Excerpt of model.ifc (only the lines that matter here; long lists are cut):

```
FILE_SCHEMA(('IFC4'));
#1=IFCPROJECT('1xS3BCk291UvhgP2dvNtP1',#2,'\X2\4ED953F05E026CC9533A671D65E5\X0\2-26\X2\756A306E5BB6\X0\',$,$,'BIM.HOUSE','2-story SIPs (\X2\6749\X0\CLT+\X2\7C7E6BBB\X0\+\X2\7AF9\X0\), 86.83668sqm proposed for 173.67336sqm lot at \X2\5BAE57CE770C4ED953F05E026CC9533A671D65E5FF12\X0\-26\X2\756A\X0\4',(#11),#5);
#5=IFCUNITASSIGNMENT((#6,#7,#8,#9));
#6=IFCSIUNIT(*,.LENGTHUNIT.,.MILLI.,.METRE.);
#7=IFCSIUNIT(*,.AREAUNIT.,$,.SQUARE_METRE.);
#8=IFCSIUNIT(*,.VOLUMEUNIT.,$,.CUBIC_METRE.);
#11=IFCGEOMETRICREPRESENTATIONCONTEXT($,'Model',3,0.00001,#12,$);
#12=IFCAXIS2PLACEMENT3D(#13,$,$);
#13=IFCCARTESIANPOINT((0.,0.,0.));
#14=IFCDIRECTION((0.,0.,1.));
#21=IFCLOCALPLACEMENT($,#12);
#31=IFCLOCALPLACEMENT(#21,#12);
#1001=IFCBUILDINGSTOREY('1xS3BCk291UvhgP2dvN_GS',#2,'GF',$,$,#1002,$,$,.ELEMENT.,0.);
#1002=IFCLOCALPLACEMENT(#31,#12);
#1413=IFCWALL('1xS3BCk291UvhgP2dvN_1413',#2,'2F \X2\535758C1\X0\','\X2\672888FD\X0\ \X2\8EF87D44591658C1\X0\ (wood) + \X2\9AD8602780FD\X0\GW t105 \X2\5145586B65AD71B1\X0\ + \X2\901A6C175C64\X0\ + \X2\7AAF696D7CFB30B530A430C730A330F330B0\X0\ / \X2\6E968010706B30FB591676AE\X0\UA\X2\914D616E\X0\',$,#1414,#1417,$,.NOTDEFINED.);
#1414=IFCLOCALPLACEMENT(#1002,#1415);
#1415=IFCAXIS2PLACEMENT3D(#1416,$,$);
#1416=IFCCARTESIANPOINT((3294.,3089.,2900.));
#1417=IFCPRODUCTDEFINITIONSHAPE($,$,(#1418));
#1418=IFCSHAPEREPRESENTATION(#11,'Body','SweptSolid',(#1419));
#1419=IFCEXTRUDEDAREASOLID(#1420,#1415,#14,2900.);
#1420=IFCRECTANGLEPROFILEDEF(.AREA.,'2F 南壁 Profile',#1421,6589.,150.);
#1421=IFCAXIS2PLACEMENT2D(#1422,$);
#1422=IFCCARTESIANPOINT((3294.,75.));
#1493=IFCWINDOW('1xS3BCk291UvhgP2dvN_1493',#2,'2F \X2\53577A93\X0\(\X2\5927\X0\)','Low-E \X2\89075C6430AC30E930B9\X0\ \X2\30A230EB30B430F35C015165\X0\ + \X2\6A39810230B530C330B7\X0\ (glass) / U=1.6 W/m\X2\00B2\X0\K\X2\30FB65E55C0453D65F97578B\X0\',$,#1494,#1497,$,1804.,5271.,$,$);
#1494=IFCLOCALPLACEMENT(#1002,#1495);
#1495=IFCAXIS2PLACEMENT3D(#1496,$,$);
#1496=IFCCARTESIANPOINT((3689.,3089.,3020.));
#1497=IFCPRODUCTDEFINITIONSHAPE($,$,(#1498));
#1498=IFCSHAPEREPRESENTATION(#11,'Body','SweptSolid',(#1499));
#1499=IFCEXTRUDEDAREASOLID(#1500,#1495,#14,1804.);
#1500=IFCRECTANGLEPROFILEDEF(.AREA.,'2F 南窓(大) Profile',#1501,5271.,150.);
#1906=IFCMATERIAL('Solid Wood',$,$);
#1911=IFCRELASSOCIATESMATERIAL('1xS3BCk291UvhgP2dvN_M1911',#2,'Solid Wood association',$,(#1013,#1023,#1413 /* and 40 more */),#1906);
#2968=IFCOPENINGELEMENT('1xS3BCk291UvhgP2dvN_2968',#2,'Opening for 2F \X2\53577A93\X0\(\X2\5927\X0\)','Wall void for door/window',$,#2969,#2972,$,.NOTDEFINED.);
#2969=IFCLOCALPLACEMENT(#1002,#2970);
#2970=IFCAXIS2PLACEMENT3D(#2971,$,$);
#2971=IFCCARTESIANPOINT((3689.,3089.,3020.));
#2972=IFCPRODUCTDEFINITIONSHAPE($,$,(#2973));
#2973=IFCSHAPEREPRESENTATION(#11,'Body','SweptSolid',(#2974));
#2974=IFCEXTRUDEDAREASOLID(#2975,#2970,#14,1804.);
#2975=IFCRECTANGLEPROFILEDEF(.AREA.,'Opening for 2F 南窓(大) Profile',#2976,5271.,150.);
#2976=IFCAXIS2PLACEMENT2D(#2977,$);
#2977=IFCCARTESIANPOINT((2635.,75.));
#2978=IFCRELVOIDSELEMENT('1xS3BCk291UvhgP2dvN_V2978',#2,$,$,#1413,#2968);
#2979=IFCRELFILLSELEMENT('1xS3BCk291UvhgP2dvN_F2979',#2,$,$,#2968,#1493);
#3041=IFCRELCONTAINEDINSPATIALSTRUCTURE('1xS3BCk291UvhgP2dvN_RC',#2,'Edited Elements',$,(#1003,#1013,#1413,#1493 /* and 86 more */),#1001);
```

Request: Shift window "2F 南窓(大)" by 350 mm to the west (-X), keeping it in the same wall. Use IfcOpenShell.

```python
import ifcopenshell
import ifcopenshell.api.geometry
import ifcopenshell.util.placement

model = ifcopenshell.open("model.ifc")

window = model.by_guid("1xS3BCk291UvhgP2dvN_1493")
opening = window.FillsVoids[0].RelatingOpeningElement
wall = opening.VoidsElements[0].RelatingBuildingElement

wall_matrix = ifcopenshell.util.placement.get_local_placement(wall.ObjectPlacement)
shift = wall_matrix[:3, 0] * -350.0
before = ifcopenshell.util.placement.get_local_placement(window.ObjectPlacement)[:3, 3].copy()

# The window is not placed relative to its opening, so move both.
for product in (opening, window):
    matrix = ifcopenshell.util.placement.get_local_placement(product.ObjectPlacement)
    matrix[:3, 3] += shift
    ifcopenshell.api.geometry.edit_object_placement(model, product=product, matrix=matrix, is_si=False)

after = ifcopenshell.util.placement.get_local_placement(window.ObjectPlacement)[:3, 3]
print("window moved by", (after - before).round(3) + 0.0)

model.write("model-out.ifc")
```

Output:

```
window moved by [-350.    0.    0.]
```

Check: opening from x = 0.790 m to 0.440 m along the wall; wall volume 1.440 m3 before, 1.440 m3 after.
